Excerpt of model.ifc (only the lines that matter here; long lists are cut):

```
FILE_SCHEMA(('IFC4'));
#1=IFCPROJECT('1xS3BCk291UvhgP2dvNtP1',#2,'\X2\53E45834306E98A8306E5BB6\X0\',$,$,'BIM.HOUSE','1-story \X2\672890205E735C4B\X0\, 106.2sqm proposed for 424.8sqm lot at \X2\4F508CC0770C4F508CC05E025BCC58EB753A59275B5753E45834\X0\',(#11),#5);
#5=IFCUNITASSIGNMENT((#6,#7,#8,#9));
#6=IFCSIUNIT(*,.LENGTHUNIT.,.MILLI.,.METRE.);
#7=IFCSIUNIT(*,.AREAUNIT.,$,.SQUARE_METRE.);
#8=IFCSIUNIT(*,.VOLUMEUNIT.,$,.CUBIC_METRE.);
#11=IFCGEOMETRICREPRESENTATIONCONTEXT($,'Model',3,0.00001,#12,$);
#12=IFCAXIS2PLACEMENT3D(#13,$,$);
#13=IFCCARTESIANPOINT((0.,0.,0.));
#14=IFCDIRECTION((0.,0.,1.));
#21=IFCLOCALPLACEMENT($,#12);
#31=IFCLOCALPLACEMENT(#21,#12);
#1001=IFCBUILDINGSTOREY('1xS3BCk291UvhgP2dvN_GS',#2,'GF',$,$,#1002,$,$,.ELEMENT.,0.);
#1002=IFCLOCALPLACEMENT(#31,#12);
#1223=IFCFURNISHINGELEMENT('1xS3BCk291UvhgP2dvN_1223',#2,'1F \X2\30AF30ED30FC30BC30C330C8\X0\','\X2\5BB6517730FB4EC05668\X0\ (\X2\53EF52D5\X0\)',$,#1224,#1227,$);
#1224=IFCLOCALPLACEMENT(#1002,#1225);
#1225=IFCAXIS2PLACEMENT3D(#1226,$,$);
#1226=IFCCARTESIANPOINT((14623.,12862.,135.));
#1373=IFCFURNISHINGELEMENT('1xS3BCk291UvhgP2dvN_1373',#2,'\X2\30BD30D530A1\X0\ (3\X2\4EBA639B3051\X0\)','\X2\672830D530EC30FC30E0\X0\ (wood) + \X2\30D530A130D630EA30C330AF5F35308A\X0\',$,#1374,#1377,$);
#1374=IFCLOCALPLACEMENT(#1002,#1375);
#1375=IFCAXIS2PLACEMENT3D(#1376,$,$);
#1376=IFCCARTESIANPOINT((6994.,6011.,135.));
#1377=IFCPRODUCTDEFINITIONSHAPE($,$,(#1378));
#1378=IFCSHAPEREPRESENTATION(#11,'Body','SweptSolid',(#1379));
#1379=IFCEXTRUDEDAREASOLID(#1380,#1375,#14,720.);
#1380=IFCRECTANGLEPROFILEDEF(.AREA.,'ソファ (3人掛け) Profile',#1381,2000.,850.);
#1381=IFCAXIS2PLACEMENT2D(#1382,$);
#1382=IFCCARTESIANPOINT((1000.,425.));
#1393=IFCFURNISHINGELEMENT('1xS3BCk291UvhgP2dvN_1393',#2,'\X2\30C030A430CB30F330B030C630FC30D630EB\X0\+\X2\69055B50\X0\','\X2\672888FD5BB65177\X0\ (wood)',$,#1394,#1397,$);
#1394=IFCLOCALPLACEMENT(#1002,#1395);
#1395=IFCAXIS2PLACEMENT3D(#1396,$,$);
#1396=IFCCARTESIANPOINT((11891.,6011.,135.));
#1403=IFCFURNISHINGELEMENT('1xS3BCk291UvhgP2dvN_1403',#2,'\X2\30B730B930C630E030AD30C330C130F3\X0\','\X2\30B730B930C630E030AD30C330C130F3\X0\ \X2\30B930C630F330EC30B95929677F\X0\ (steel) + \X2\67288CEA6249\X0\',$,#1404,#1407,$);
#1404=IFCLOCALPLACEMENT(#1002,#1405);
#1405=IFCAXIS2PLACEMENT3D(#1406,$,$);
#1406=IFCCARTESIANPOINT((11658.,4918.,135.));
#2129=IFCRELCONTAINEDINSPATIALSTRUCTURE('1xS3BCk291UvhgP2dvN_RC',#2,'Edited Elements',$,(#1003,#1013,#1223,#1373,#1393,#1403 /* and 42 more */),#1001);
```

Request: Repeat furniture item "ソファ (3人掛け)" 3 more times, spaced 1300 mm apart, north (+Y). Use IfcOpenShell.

```python
import numpy as np
import ifcopenshell
import ifcopenshell.api.geometry
import ifcopenshell.api.root
import ifcopenshell.util.element
import ifcopenshell.util.placement
import ifcopenshell.util.unit

model = ifcopenshell.open("model.ifc")
unit_scale = ifcopenshell.util.unit.calculate_unit_scale(model)


def reuse_history(source, copy):
    """copy_class also copies each property set's owner history, people and application; keep the originals."""
    for rel in copy.IsDefinedBy:
        if rel.is_a("IfcRelDefinesByProperties") and (history := rel.RelatingPropertyDefinition.OwnerHistory):
            rel.RelatingPropertyDefinition.OwnerHistory = source.OwnerHistory
            ifcopenshell.util.element.remove_deep2(model, history)


source = model.by_guid("1xS3BCk291UvhgP2dvN_1373")
base = ifcopenshell.util.placement.get_local_placement(source.ObjectPlacement)
step = np.array([0.0, 1.0, 0.0]) * 1.3 / unit_scale

for i in range(1, 4):
    copy = ifcopenshell.api.root.copy_class(model, product=source)
    copy.Representation = ifcopenshell.util.element.copy_deep(
        model, source.Representation, exclude=["IfcGeometricRepresentationContext", "IfcRepresentationMap"]
    )
    reuse_history(source, copy)
    matrix = base.copy()
    matrix[:3, 3] += i * step
    print("added at", matrix[:3, 3].round(3) + 0.0)
    ifcopenshell.api.geometry.edit_object_placement(model, product=copy, matrix=matrix, is_si=False)

model.write("model_updated.ifc")
```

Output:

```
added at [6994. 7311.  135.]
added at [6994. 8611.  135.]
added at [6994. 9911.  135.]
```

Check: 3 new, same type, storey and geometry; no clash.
